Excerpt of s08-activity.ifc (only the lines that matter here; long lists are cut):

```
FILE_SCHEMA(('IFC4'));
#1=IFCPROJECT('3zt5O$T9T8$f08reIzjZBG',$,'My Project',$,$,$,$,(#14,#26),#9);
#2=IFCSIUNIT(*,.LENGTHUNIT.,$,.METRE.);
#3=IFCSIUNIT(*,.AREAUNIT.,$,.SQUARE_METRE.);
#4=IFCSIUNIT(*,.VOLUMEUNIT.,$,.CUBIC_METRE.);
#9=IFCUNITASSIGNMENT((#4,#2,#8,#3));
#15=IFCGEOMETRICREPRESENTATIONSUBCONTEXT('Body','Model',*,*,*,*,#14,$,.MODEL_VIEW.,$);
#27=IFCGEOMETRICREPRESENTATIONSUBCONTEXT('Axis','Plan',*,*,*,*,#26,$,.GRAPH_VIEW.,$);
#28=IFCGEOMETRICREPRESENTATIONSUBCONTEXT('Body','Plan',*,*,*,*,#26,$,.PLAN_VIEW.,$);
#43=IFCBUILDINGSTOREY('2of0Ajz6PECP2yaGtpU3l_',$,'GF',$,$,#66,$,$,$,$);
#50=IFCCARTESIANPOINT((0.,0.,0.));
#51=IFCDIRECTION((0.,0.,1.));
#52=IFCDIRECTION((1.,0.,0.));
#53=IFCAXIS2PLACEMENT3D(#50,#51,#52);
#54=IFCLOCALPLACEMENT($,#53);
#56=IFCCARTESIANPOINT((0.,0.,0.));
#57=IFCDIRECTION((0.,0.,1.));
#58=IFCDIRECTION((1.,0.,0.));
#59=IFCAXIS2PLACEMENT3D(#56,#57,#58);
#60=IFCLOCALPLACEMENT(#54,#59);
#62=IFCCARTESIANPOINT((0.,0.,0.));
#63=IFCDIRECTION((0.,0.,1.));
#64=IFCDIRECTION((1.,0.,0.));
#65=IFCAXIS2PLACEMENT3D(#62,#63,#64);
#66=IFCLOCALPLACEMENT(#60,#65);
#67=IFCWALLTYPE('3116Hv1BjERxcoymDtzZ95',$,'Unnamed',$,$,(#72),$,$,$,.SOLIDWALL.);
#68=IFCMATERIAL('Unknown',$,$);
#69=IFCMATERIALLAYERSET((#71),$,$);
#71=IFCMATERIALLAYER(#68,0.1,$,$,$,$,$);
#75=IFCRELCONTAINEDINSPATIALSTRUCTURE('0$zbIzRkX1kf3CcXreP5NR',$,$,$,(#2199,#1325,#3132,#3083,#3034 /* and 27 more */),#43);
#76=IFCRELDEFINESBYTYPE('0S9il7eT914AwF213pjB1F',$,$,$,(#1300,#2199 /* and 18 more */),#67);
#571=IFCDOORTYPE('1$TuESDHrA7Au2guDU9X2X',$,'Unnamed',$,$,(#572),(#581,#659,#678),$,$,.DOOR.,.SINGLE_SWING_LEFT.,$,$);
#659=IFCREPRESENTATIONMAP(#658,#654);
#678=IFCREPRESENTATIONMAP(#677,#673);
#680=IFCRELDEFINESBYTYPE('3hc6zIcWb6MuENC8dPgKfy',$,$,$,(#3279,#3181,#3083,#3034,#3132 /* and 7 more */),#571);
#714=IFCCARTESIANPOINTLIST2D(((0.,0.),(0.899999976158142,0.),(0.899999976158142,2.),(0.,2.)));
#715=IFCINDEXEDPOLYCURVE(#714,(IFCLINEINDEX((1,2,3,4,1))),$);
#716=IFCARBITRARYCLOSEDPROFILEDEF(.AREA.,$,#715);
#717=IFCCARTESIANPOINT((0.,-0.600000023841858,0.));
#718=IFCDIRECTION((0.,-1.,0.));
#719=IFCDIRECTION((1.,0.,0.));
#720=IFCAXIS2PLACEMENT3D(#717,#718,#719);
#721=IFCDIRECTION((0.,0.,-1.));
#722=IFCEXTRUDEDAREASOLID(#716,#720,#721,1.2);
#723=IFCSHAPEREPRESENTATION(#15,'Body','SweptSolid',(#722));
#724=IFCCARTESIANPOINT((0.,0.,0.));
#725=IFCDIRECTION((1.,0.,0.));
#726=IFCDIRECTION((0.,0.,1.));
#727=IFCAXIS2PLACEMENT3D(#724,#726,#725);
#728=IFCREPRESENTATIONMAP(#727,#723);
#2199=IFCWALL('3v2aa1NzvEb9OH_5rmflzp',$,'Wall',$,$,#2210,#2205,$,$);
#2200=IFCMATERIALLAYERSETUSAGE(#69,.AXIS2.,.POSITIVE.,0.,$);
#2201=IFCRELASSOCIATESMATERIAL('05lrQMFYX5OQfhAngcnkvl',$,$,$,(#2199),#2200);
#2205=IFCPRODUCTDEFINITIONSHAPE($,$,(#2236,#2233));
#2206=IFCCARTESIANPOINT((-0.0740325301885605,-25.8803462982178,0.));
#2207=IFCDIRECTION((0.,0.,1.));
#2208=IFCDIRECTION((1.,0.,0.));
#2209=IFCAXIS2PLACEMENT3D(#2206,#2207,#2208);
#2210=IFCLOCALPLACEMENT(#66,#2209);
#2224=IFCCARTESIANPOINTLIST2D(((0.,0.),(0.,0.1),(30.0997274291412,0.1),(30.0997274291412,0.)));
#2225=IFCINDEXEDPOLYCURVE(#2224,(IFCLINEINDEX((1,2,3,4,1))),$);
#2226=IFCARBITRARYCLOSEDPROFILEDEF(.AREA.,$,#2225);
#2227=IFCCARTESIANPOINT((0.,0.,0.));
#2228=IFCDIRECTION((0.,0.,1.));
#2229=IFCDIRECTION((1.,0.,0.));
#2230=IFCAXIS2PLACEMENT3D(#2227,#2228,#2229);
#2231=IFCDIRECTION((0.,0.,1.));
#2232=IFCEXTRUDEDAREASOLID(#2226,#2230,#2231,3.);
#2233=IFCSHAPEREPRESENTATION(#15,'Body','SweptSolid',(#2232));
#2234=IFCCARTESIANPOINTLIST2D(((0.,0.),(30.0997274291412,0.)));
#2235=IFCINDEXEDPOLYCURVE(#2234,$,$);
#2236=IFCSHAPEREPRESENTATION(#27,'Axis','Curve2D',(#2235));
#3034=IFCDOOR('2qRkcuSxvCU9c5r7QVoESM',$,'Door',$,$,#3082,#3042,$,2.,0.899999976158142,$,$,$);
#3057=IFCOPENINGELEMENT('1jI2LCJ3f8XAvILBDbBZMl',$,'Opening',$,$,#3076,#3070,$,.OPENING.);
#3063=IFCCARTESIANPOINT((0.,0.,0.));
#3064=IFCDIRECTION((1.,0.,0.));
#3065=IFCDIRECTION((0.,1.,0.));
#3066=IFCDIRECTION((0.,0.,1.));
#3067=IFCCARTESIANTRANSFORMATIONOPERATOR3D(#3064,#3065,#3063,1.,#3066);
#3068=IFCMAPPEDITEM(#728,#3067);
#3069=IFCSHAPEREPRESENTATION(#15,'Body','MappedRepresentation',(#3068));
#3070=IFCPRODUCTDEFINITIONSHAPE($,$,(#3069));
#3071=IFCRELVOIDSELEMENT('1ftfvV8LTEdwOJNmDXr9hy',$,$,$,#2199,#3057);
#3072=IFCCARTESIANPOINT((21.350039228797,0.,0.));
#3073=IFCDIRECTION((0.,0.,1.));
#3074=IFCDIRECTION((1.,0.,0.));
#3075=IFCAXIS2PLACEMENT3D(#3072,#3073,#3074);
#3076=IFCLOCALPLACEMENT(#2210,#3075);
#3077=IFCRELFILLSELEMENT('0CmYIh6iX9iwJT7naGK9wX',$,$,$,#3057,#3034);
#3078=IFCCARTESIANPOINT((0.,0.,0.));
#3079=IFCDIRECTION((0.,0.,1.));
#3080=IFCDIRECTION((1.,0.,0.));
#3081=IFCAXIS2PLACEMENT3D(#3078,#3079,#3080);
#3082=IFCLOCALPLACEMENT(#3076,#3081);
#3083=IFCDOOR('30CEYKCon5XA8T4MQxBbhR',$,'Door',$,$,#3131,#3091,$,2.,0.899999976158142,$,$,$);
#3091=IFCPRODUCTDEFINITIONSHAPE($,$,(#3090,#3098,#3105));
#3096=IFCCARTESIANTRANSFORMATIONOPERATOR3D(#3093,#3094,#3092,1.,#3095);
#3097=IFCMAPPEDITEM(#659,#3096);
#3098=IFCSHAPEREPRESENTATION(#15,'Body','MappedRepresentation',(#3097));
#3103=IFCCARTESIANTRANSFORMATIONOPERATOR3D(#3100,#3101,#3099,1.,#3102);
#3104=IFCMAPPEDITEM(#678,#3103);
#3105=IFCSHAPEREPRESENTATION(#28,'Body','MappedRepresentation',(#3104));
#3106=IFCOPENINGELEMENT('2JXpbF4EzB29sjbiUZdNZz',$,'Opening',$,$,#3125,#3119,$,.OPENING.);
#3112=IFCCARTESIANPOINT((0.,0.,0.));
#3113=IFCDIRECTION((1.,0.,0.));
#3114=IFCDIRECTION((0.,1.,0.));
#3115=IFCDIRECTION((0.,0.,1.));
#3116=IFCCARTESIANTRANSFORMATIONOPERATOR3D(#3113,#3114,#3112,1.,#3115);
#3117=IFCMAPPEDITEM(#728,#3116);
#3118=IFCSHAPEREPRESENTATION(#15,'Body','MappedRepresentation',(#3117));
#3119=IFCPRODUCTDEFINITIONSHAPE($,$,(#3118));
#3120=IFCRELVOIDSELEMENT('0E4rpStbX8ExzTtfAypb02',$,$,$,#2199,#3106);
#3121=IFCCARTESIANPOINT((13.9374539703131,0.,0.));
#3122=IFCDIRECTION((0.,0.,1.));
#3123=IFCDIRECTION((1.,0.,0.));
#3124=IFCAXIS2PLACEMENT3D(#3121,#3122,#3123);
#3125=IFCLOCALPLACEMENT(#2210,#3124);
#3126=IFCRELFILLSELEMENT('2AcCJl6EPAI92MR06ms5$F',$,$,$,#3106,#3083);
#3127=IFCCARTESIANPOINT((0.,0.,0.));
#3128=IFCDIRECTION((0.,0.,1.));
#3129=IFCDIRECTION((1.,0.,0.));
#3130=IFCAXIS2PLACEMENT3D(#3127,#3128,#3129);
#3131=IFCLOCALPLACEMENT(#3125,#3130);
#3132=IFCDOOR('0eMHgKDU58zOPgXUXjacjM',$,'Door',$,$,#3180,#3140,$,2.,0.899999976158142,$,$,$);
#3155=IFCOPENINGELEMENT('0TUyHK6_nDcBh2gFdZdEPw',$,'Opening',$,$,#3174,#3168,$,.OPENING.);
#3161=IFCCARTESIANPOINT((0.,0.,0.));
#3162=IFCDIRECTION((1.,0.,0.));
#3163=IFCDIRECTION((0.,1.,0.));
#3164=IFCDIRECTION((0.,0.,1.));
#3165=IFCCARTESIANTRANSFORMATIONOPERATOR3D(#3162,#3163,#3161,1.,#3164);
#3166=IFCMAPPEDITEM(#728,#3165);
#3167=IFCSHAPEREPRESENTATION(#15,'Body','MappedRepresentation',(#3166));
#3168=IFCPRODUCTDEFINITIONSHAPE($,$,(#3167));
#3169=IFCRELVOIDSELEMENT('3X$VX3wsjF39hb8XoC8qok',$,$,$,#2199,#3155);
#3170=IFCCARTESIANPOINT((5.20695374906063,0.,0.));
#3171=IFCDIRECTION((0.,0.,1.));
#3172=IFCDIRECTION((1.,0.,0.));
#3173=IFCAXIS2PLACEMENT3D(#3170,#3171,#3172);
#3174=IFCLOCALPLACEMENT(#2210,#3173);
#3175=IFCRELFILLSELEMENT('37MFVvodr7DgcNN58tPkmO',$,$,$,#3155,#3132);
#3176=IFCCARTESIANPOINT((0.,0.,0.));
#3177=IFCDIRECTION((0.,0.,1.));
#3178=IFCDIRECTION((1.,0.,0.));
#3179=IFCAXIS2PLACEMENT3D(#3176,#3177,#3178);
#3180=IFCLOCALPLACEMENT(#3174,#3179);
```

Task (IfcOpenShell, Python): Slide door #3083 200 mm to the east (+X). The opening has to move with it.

```python
import ifcopenshell
import ifcopenshell.api.geometry
import ifcopenshell.util.placement
import ifcopenshell.util.unit

model = ifcopenshell.open("s08-activity.ifc")
unit_scale = ifcopenshell.util.unit.calculate_unit_scale(model)

door = model.by_guid("30CEYKCon5XA8T4MQxBbhR")
opening = door.FillsVoids[0].RelatingOpeningElement
wall = opening.VoidsElements[0].RelatingBuildingElement

wall_matrix = ifcopenshell.util.placement.get_local_placement(wall.ObjectPlacement)
shift = wall_matrix[:3, 0] * 0.2 / unit_scale
before = ifcopenshell.util.placement.get_local_placement(door.ObjectPlacement)[:3, 3].copy()

# The door is placed relative to its opening, so it follows when the opening moves.
matrix = ifcopenshell.util.placement.get_local_placement(opening.ObjectPlacement)
matrix[:3, 3] += shift
ifcopenshell.api.geometry.edit_object_placement(
    model, product=opening, matrix=matrix, is_si=False, should_transform_children=True
)

after = ifcopenshell.util.placement.get_local_placement(door.ObjectPlacement)[:3, 3]
print("door moved by", (after - before).round(3) + 0.0)

model.write("s08-activity_rev.ifc")
```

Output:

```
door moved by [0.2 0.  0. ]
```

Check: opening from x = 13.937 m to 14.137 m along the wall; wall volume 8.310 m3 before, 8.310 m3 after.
